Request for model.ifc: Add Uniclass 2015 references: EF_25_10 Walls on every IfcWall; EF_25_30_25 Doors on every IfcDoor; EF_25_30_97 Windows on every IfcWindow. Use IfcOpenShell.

First a look at what the model holds.

```python
import ifcopenshell

model = ifcopenshell.open("model.ifc")
print(model.schema)
print("classifications:", [c.Name for c in model.by_type("IfcClassification")])
for ifc_class in ("IfcDoor", "IfcRoof", "IfcStair", "IfcWall", "IfcWindow"):
    print(ifc_class, len(model.by_type(ifc_class)))
```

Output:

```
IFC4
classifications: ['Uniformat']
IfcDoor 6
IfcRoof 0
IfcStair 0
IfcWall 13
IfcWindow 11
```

```python
import ifcopenshell
import ifcopenshell.api.classification

model = ifcopenshell.open("model.ifc")

system = ifcopenshell.api.classification.add_classification(model, classification="Uniclass 2015")

codes = {
    "IfcWall": ("EF_25_10", "Walls"),
    "IfcDoor": ("EF_25_30_25", "Doors"),
    "IfcWindow": ("EF_25_30_97", "Windows"),
}
for ifc_class, (code, name) in codes.items():
    products = model.by_type(ifc_class)
    ifcopenshell.api.classification.add_reference(
        model, products=products, classification=system, identification=code, name=name
    )
    print(code, len(products))

model.write("model-out.ifc")
```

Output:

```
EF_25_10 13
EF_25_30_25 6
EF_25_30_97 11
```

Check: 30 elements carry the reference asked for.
